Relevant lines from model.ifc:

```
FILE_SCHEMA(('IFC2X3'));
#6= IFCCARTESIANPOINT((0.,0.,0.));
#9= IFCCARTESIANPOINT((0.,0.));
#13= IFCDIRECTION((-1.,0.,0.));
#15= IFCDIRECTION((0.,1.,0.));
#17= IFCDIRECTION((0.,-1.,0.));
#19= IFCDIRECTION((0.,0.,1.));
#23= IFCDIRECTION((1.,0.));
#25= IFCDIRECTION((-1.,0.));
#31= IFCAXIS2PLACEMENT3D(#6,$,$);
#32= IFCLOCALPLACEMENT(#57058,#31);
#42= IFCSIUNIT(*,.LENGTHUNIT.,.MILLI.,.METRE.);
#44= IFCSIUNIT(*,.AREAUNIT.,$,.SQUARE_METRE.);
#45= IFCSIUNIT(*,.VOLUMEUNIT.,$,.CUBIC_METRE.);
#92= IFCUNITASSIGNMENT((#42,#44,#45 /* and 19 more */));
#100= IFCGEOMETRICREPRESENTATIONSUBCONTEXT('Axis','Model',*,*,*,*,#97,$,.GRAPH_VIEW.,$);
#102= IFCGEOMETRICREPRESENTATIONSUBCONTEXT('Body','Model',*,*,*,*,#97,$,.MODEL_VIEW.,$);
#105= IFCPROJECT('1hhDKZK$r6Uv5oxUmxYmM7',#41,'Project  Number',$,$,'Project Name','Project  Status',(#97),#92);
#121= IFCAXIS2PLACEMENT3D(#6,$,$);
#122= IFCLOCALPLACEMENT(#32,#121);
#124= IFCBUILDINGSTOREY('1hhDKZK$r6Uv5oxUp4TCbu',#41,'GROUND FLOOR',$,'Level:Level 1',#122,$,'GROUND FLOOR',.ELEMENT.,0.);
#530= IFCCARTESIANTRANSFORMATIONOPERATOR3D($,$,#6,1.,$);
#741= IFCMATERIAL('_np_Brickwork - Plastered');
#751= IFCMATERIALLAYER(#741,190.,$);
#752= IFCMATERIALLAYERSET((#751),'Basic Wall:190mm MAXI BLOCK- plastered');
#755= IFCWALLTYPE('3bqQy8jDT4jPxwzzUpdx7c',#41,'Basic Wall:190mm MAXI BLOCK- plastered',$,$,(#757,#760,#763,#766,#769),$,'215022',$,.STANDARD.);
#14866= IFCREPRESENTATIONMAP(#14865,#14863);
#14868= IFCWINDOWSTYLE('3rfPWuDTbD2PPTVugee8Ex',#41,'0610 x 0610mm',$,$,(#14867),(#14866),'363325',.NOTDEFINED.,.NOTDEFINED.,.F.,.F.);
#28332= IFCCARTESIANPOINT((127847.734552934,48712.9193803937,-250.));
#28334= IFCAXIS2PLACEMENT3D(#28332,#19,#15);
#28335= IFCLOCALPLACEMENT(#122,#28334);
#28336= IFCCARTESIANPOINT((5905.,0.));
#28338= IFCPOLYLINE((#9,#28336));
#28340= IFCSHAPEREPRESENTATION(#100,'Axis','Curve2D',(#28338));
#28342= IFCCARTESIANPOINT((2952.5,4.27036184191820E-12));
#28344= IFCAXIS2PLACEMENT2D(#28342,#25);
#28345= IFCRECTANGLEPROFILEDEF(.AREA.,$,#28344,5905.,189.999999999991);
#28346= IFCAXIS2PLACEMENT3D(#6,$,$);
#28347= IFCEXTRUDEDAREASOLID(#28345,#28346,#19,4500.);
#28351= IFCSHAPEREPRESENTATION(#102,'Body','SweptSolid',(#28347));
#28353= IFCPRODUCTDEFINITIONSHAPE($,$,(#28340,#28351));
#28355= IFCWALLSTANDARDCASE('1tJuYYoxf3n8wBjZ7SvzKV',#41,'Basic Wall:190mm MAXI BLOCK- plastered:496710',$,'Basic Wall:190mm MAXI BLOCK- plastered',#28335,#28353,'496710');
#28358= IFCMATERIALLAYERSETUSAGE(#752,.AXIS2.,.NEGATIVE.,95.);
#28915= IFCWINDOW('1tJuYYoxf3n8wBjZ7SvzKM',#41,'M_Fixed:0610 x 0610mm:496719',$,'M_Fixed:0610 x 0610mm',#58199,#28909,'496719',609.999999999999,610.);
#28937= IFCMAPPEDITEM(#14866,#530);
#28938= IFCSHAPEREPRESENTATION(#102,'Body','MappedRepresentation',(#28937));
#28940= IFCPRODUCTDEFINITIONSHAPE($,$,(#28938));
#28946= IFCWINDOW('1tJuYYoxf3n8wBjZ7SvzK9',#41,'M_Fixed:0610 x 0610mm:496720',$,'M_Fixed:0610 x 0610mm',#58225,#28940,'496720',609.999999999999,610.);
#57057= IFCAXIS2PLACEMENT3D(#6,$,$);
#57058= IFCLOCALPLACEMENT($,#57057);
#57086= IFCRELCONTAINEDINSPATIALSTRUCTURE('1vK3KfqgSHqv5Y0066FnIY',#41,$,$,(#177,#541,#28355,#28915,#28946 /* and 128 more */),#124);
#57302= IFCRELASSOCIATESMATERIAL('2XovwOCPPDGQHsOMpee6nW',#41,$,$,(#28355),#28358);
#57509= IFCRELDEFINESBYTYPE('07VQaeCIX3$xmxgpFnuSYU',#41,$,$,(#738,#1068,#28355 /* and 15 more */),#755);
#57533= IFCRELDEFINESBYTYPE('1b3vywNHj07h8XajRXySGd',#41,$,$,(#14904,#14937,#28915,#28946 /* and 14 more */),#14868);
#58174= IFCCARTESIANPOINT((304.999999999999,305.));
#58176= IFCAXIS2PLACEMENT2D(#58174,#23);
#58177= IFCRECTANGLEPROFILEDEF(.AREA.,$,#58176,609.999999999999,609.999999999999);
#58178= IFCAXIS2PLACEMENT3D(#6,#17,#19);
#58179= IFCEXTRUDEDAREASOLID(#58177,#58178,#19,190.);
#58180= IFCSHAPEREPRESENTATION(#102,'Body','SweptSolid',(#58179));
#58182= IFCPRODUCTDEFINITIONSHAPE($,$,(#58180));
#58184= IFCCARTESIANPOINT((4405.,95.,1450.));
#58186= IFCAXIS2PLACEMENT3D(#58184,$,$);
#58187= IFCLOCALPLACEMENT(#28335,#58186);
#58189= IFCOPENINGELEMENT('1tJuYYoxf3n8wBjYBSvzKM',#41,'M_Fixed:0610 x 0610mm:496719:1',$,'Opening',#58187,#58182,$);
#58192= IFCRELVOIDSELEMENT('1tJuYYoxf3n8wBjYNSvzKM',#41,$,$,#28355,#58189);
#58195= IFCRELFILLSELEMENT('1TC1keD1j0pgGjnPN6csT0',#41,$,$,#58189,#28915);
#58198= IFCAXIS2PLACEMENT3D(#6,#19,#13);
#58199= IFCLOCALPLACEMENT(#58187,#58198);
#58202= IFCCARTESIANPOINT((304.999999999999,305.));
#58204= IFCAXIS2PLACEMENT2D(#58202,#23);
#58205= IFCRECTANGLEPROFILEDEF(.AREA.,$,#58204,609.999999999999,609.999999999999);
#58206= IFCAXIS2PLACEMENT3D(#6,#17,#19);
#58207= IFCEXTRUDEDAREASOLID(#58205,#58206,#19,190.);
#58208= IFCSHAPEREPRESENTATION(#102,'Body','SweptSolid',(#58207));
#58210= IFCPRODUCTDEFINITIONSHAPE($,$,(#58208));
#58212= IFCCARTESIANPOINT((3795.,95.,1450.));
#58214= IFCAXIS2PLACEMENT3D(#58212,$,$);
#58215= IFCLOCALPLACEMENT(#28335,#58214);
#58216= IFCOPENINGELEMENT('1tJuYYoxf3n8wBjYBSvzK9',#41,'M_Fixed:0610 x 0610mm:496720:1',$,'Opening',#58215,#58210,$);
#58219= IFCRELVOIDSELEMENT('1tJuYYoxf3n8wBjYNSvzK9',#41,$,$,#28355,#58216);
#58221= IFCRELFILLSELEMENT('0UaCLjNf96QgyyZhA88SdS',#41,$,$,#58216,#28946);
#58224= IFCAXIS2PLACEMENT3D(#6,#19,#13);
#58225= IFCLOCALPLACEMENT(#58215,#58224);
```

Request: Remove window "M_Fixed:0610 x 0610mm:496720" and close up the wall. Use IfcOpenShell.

```python
import ifcopenshell
import ifcopenshell.api.feature
import ifcopenshell.api.root
import ifcopenshell.geom
import ifcopenshell.util.shape

model = ifcopenshell.open("model.ifc")
settings = ifcopenshell.geom.settings()


def volume(element):
    """Net volume in cubic metres, openings subtracted."""
    shape = ifcopenshell.geom.create_shape(settings, element)
    return ifcopenshell.util.shape.get_volume(shape.geometry)


window = model.by_guid("1tJuYYoxf3n8wBjZ7SvzK9")
opening = window.FillsVoids[0].RelatingOpeningElement
wall = opening.VoidsElements[0].RelatingBuildingElement
before = volume(wall)

ifcopenshell.api.root.remove_product(model, product=window)
ifcopenshell.api.feature.remove_feature(model, feature=opening)

after = volume(wall)

print(f"wall volume {before:.3f} -> {after:.3f} m3")

model.write("model_v2.ifc")
```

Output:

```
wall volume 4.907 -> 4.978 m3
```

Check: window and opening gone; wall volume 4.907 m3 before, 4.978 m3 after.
